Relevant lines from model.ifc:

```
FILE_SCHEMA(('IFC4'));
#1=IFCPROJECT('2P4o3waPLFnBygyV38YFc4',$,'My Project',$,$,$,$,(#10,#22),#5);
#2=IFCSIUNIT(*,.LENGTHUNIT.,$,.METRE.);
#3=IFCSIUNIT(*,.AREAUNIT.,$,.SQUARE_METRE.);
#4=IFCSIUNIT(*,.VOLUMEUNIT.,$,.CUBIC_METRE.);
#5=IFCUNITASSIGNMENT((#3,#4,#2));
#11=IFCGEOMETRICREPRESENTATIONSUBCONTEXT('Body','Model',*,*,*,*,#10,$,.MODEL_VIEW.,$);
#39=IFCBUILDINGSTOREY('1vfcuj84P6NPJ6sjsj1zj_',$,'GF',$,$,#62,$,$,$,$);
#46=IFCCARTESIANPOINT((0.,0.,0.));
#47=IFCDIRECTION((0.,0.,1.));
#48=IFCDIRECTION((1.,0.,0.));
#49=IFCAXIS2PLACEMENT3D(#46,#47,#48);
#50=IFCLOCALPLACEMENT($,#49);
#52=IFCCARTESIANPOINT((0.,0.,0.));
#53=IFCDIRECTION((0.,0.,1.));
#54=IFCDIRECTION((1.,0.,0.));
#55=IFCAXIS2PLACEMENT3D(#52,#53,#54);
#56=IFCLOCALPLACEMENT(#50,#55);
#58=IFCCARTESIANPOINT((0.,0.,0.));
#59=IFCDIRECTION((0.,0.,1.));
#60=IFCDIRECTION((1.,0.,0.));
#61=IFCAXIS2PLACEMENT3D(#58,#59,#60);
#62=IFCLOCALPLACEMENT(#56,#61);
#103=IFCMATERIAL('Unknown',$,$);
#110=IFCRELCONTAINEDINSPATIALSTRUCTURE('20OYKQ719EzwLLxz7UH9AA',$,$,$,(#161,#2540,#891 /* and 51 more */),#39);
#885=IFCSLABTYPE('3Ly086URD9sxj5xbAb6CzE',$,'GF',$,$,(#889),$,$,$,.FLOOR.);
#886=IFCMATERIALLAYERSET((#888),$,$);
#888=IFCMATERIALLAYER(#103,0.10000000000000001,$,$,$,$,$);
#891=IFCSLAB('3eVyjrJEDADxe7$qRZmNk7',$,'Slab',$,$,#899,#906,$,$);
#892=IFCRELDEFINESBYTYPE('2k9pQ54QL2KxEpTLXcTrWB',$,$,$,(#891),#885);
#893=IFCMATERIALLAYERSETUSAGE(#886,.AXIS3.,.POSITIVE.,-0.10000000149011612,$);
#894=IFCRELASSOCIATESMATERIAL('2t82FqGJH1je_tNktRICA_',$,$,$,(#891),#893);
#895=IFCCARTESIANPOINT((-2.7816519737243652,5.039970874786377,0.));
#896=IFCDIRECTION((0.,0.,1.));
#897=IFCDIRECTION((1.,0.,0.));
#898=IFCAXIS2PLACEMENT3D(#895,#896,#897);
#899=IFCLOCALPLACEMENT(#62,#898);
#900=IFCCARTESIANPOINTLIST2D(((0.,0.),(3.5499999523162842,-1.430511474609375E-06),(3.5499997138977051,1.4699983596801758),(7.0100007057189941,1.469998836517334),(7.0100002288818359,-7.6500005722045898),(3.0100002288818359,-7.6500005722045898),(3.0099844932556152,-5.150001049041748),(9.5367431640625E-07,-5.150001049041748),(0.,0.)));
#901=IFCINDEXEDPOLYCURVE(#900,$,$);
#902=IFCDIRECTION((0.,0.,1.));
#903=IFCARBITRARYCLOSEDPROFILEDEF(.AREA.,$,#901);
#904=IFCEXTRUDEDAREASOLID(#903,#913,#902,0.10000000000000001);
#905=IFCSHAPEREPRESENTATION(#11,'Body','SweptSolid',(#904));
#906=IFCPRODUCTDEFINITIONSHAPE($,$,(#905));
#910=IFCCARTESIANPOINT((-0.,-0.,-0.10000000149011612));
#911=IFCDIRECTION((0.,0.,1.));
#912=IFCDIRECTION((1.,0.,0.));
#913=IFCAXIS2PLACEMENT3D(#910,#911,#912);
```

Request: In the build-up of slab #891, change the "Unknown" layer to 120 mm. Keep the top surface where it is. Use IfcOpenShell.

```python
import ifcopenshell
import ifcopenshell.util.element
import ifcopenshell.util.representation

model = ifcopenshell.open("model.ifc")

layer_set = model.by_id(886)
layer = next(l for l in layer_set.MaterialLayers if l.Material and l.Material.Name == "Unknown")
change = 0.12 - layer.LayerThickness
layer.LayerThickness += change

# Geometry does not follow the layer set by itself.
slabs = [e for e in ifcopenshell.util.element.get_elements_by_material(model, layer_set) if e.is_a("IfcSlab")]
for slab in sorted(slabs, key=lambda e: e.id()):
    body = ifcopenshell.util.representation.get_representation(slab, "Model", "Body")
    solid = body.Items[0]
    old_depth = solid.Depth
    solid.Depth += change
    # Extruded upwards: lower the start of the extrusion so the top stays.
    x, y, z = solid.Position.Location.Coordinates
    solid.Position.Location = model.createIfcCartesianPoint((x, y, z - change))
    print(slab.id(), f"{old_depth:g} -> {solid.Depth:g}")

# The layers are counted up from the underside, which has moved.
for usage in {ifcopenshell.util.element.get_material(slab) for slab in slabs}:
    usage.OffsetFromReferenceLine -= change

model.write("model_rev.ifc")
```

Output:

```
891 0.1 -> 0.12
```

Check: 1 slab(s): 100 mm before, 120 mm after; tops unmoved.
